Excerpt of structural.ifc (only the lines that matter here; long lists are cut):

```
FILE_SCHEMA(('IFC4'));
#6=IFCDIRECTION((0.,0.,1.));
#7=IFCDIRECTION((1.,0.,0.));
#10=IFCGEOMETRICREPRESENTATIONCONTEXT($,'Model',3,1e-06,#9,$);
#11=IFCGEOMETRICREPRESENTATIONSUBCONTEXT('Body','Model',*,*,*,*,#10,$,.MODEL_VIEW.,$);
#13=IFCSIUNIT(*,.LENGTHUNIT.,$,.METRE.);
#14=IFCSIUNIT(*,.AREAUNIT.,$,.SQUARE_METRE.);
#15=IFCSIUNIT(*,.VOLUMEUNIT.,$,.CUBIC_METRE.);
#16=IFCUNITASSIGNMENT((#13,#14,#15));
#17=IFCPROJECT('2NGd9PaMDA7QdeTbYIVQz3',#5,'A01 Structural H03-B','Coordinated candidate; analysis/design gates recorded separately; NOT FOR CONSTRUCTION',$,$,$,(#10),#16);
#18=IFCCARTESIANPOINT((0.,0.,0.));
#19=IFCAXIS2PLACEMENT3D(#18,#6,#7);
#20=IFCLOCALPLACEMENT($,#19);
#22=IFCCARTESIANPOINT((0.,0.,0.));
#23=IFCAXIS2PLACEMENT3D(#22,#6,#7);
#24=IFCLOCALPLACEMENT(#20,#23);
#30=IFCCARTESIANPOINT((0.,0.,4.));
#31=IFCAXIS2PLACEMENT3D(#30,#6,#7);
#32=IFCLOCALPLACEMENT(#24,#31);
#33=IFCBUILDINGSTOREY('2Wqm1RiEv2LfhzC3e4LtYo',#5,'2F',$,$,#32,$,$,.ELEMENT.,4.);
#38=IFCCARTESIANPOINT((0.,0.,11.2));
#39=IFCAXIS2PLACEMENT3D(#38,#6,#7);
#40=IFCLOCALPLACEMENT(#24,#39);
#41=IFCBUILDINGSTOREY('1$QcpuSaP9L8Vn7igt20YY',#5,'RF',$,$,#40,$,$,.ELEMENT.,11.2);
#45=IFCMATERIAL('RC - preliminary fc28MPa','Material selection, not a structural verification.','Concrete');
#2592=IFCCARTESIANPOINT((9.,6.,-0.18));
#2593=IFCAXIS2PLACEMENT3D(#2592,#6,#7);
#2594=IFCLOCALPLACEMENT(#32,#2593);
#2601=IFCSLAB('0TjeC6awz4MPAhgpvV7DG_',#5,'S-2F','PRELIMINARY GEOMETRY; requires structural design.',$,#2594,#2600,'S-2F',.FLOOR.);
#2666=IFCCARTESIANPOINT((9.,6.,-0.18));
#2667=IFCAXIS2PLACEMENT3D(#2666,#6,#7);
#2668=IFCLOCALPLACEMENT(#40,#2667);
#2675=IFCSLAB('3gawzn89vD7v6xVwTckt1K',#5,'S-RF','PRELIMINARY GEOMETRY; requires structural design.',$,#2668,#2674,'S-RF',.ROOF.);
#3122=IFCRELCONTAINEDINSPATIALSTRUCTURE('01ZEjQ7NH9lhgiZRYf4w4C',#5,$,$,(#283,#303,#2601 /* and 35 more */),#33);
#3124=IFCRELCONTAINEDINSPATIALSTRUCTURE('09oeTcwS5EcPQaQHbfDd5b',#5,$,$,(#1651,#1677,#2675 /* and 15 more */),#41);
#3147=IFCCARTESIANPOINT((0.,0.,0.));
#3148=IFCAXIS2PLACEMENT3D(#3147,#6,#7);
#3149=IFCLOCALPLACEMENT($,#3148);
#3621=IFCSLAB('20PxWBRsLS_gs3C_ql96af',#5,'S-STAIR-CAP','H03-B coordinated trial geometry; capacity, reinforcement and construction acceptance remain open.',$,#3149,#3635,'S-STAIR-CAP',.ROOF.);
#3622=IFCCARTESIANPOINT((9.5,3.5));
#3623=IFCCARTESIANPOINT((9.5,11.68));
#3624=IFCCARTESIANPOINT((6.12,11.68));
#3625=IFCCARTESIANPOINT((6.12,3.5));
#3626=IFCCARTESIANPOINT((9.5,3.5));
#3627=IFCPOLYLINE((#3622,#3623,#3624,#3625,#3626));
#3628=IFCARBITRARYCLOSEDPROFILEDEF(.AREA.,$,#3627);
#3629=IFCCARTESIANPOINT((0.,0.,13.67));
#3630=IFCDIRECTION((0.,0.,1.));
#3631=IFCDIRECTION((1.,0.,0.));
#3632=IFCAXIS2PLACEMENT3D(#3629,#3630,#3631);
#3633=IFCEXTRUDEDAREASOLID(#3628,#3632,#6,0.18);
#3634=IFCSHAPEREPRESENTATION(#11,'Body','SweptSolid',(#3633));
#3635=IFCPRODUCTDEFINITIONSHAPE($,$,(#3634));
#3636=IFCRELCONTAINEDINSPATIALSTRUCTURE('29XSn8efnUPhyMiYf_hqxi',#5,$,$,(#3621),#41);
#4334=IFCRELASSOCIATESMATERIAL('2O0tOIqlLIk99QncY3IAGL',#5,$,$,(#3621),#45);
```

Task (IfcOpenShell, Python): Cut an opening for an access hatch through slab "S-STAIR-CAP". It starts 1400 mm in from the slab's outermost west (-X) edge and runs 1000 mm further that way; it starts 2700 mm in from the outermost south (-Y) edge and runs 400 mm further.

```python
import numpy as np
import ifcopenshell
import ifcopenshell.api.feature
import ifcopenshell.api.geometry
import ifcopenshell.api.root
import ifcopenshell.geom
import ifcopenshell.util.placement
import ifcopenshell.util.representation
import ifcopenshell.util.shape
import ifcopenshell.util.unit

model = ifcopenshell.open("structural.ifc")
unit_scale = ifcopenshell.util.unit.calculate_unit_scale(model)
settings = ifcopenshell.geom.settings()


def volume(element):
    """Net volume in cubic metres, openings subtracted."""
    shape = ifcopenshell.geom.create_shape(settings, element)
    return ifcopenshell.util.shape.get_volume(shape.geometry)


slab = model.by_guid("20PxWBRsLS_gs3C_ql96af")
before = volume(slab)

# Extent in the slab's own axes, in metres. The edges named are its -X and -Y sides.
slab_shape = ifcopenshell.geom.create_shape(settings, slab)
vertices = ifcopenshell.util.shape.get_vertices(slab_shape.geometry)
x_min, y_min, bottom = vertices.min(axis=0)
top = vertices[:, 2].max()

opening = ifcopenshell.api.root.create_entity(model, ifc_class="IfcOpeningElement", name="Access hatch opening", predefined_type="OPENING")
context = ifcopenshell.util.representation.get_context(model, "Model", "Body", "MODEL_VIEW")
width, depth = 1, 0.4
outline = [(0.0, 0.0), (width, 0.0), (width, depth), (0.0, depth), (0.0, 0.0)]
# Overshoot both faces by 50 mm so the cut is clean.
shape = ifcopenshell.api.geometry.add_slab_representation(
    model, context=context, depth=top - bottom + 0.1, polyline=outline
)
ifcopenshell.api.geometry.assign_representation(model, product=opening, representation=shape)

matrix = ifcopenshell.util.placement.get_local_placement(slab.ObjectPlacement)
matrix[:, 3] = matrix @ np.append(np.array([x_min + 1.4, y_min + 2.7, bottom - 0.05]) / unit_scale, 1.0)
ifcopenshell.api.geometry.edit_object_placement(model, product=opening, matrix=matrix, is_si=False)
ifcopenshell.api.feature.add_feature(model, feature=opening, element=slab)

after = volume(slab)

print(f"slab volume {before:.3f} -> {after:.3f} m3")

model.write("structural_rev.ifc")
```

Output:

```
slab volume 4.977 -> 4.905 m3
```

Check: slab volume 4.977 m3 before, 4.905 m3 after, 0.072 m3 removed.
